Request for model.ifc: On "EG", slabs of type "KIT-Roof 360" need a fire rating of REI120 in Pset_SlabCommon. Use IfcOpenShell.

First a look at what the model holds.

```python
import ifcopenshell
import ifcopenshell.util.element

model = ifcopenshell.open("model.ifc")
print(model.schema)
storey = next(s for s in model.by_type("IfcBuildingStorey") if s.Name == "EG")
slabs = [e for e in ifcopenshell.util.element.get_decomposition(storey) if e.is_a("IfcSlab")]
seen = {}
for e in slabs:
    element_type = ifcopenshell.util.element.get_type(e)
    key = (element_type.Name if element_type != e and element_type else None, ifcopenshell.util.element.get_pset(e, "Pset_SlabCommon", "FireRating"))
    seen[key] = seen.get(key, 0) + 1
for (name, value), count in sorted(seen.items(), key=str):
    print(count, "x", name, "|", value)
```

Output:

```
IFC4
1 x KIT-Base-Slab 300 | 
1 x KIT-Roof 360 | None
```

```python
import ifcopenshell
import ifcopenshell.api.pset
import ifcopenshell.util.element

model = ifcopenshell.open("model.ifc")

storey = next(s for s in model.by_type("IfcBuildingStorey") if s.Name == "EG")
slabs = [e for e in ifcopenshell.util.element.get_decomposition(storey) if e.is_a("IfcSlab")]

count = 0
for e in slabs:
    element_type = ifcopenshell.util.element.get_type(e)
    if element_type in (None, e) or element_type.Name != "KIT-Roof 360":
        continue
    # add_pset returns the element's existing set when there is one.
    pset = ifcopenshell.api.pset.add_pset(model, product=e, name="Pset_SlabCommon")
    ifcopenshell.api.pset.edit_pset(model, pset=pset, properties={"FireRating": "REI120"})
    count += 1

print(count, "slabs updated")

model.write("model_rev.ifc")
```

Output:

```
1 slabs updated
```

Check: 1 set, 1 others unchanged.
